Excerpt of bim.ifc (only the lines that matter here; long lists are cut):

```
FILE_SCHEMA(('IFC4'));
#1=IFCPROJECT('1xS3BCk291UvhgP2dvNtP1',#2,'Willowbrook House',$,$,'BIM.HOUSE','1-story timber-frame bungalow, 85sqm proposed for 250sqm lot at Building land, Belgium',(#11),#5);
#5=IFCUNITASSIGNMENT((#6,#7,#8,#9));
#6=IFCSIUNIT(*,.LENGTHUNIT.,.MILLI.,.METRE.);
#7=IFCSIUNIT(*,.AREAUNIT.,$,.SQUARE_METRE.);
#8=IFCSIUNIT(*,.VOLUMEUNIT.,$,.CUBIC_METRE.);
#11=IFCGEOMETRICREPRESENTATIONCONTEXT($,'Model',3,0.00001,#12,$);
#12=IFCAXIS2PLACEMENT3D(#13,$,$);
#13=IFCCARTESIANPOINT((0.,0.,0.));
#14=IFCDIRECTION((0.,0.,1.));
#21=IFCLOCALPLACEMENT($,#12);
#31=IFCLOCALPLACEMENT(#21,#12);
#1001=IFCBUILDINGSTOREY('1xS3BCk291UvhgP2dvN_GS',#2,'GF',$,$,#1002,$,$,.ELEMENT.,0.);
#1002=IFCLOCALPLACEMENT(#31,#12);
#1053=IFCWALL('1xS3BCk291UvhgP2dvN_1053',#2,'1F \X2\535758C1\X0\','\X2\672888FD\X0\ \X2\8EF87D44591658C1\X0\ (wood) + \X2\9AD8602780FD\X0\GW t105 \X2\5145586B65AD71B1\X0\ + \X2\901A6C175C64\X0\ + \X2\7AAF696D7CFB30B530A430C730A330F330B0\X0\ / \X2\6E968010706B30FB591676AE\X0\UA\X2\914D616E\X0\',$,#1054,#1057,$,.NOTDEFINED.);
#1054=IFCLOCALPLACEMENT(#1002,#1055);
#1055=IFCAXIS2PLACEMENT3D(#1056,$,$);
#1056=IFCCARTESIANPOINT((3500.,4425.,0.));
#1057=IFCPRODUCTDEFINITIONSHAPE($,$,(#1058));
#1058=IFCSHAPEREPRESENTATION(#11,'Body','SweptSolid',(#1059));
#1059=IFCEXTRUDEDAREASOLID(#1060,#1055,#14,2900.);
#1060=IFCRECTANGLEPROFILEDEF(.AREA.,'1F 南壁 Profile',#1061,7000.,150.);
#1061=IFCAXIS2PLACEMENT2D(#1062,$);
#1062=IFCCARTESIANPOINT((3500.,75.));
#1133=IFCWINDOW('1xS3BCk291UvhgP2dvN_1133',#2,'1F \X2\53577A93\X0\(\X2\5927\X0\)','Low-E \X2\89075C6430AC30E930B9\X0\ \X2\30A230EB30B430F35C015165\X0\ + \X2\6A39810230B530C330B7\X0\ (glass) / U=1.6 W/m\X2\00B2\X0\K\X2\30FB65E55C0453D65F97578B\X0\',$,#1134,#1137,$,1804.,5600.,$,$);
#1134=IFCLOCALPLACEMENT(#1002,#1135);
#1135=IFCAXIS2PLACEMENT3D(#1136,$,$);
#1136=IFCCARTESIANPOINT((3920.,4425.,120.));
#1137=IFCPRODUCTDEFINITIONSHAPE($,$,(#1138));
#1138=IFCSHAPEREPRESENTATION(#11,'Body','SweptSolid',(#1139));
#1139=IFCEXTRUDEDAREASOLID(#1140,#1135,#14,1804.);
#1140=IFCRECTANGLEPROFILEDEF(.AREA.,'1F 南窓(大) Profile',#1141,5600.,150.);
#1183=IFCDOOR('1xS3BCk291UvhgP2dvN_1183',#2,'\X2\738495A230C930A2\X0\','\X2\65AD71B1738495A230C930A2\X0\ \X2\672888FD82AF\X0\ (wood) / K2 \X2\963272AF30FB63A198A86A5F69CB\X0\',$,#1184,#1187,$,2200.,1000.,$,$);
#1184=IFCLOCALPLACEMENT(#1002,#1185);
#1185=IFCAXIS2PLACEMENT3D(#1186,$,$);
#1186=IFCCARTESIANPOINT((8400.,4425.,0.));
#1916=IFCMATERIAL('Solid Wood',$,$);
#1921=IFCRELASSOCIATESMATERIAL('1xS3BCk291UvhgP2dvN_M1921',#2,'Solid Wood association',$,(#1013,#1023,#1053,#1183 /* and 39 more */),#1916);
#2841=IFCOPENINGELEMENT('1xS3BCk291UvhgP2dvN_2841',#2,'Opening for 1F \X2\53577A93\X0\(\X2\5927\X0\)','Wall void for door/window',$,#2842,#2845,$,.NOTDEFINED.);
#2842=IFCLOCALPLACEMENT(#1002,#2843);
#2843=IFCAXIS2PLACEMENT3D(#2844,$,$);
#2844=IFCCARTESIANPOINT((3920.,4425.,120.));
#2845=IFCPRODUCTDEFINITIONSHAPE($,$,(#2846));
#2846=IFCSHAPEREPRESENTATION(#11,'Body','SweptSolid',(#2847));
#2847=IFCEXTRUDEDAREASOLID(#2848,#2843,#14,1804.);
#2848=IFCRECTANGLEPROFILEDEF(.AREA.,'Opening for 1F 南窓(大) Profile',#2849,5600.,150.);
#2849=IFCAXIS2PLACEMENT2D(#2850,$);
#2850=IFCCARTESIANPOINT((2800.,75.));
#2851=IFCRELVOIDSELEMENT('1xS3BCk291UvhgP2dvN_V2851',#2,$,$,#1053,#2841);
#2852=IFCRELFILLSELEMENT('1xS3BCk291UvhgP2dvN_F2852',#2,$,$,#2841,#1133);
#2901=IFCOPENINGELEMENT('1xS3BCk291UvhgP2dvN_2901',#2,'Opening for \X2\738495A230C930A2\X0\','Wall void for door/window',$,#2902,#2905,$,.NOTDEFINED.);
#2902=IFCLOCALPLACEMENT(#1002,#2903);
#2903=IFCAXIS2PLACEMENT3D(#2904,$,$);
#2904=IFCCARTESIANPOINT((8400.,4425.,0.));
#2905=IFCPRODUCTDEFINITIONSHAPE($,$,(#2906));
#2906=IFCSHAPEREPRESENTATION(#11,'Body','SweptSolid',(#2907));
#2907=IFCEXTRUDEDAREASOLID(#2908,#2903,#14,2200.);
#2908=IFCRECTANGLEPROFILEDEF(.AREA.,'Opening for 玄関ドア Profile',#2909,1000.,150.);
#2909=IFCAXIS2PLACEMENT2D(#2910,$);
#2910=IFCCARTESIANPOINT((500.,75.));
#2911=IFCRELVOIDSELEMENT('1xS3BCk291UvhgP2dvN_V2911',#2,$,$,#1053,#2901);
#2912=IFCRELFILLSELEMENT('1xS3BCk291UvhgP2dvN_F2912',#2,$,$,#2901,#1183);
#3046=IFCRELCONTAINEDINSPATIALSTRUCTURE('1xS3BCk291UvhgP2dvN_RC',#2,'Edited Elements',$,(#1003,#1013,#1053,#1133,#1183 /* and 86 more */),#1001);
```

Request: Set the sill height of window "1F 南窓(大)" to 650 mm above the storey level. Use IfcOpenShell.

```python
import numpy as np
import ifcopenshell
import ifcopenshell.api.geometry
import ifcopenshell.geom
import ifcopenshell.util.element
import ifcopenshell.util.placement
import ifcopenshell.util.shape
import ifcopenshell.util.unit

model = ifcopenshell.open("bim.ifc")
unit_scale = ifcopenshell.util.unit.calculate_unit_scale(model)

window = model.by_guid("1xS3BCk291UvhgP2dvN_1133")
opening = window.FillsVoids[0].RelatingOpeningElement
storey = ifcopenshell.util.element.get_container(window, ifc_class="IfcBuildingStorey")
level = ifcopenshell.util.placement.get_local_placement(storey.ObjectPlacement)[2, 3]

# The opening's origin need not be at the sill, so measure its lowest point.
shape = ifcopenshell.geom.create_shape(ifcopenshell.geom.settings(), opening)
bottom = ifcopenshell.util.shape.get_shape_bottom_elevation(shape, shape.geometry) / unit_scale
dz = level + 0.65 / unit_scale - bottom

shift = np.array([0.0, 0.0, dz])
# The window is not placed relative to its opening, so move both.
for product in (opening, window):
    matrix = ifcopenshell.util.placement.get_local_placement(product.ObjectPlacement)
    matrix[:3, 3] += shift
    ifcopenshell.api.geometry.edit_object_placement(model, product=product, matrix=matrix, is_si=False)

print(f"moved by {dz * unit_scale:+.3f} m")

model.write("bim_rev.ifc")
```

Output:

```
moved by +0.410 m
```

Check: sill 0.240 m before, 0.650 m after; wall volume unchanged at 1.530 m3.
